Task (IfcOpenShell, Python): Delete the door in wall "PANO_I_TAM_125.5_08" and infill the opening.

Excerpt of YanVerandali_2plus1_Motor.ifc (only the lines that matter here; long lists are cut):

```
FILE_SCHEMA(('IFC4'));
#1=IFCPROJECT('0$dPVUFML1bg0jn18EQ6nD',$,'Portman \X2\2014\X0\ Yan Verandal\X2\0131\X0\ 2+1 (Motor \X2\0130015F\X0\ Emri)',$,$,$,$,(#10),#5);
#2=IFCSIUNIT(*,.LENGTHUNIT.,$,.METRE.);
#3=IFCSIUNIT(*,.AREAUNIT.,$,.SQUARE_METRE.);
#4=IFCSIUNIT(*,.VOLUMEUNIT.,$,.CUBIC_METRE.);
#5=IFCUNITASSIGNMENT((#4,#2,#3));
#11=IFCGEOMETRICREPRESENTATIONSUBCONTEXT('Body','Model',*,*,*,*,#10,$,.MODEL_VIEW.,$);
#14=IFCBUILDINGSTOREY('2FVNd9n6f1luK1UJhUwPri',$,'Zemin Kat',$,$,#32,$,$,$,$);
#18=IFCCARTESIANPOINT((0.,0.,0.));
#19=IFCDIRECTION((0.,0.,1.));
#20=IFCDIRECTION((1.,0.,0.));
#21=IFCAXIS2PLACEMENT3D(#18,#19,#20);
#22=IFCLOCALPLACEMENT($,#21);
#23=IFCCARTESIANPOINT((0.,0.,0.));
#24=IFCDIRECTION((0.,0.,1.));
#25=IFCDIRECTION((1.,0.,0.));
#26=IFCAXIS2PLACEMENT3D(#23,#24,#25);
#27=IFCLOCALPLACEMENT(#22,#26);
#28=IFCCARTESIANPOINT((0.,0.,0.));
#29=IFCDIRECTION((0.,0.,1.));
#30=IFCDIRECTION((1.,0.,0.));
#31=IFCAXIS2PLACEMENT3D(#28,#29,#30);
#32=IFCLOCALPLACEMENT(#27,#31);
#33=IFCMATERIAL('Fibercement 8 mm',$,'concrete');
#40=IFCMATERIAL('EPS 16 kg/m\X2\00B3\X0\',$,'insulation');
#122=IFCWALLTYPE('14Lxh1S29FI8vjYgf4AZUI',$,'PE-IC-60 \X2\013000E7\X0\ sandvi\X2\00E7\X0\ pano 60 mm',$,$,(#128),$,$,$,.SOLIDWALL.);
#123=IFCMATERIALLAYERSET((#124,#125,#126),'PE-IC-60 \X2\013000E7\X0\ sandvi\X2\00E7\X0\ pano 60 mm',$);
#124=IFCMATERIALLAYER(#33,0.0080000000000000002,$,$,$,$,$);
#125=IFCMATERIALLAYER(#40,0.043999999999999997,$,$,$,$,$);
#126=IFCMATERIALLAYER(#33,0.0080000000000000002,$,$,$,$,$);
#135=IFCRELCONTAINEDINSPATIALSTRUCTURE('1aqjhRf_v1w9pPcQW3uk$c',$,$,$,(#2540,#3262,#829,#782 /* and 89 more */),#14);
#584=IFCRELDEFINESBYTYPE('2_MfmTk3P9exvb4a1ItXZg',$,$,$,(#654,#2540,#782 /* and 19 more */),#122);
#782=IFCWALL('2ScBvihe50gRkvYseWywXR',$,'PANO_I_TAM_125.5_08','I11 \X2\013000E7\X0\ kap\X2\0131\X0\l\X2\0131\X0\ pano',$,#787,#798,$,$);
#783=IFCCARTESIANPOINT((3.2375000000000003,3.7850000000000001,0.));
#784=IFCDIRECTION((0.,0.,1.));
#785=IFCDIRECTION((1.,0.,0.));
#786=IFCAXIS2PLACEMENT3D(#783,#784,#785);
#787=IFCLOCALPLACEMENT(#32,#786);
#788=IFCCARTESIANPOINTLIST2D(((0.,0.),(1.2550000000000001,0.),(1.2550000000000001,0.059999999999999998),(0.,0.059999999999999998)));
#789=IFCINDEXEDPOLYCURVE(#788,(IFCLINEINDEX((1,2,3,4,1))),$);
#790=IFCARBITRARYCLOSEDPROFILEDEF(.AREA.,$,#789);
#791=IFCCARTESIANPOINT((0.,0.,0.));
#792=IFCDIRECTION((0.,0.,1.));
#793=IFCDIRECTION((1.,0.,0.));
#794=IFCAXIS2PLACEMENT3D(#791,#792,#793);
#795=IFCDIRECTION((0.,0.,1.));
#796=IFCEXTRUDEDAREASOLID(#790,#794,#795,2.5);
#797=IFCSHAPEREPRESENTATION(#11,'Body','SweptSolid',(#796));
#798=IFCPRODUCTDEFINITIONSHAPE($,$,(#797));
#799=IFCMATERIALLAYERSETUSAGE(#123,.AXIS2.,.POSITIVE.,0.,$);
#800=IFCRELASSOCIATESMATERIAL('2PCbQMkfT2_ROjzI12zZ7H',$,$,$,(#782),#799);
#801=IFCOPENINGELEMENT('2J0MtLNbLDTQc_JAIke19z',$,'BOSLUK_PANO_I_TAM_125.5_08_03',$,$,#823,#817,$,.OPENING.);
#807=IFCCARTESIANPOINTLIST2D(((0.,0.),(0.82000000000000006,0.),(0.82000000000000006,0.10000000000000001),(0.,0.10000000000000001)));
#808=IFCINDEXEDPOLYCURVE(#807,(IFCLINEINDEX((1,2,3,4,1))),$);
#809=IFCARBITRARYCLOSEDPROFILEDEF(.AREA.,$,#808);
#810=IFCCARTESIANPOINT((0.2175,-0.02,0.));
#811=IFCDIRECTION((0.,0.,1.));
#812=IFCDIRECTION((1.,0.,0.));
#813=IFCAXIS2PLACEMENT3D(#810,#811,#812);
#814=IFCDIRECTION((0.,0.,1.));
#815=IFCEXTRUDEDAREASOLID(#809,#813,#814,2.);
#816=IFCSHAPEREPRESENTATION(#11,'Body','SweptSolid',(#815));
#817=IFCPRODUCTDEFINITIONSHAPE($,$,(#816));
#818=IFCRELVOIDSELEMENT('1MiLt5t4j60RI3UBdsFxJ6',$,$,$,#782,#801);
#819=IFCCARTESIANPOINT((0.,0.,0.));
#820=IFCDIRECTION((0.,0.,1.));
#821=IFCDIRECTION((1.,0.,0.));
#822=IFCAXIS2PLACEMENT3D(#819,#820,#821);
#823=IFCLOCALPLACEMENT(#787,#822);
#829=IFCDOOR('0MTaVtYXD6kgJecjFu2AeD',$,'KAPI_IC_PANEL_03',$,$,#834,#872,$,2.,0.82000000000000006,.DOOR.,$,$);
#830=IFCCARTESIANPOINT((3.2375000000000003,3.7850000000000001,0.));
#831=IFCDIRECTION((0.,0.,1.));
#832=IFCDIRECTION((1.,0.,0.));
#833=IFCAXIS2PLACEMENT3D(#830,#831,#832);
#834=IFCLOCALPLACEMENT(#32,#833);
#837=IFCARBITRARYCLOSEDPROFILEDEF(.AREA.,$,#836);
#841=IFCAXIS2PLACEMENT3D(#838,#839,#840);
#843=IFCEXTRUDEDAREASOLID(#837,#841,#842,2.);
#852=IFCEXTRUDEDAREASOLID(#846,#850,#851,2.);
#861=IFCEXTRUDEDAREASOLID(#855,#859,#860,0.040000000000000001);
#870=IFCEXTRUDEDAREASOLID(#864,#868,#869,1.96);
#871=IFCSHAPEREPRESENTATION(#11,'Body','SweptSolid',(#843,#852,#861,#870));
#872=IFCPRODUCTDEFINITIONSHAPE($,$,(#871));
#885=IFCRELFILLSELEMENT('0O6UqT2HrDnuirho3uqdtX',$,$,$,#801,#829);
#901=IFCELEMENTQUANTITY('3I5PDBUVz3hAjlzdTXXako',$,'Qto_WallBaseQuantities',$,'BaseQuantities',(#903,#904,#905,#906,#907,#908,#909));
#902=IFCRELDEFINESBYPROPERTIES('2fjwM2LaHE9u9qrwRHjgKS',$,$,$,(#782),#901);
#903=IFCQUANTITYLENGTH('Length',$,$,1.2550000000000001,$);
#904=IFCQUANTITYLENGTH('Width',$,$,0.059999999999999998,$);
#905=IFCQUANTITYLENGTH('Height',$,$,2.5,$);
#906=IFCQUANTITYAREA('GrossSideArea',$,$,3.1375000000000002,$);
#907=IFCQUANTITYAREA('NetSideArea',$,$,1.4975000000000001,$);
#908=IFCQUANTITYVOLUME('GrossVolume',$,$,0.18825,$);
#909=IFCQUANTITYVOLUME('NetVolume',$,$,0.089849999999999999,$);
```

```python
import ifcopenshell
import ifcopenshell.api.feature
import ifcopenshell.api.pset
import ifcopenshell.api.root
import ifcopenshell.geom
import ifcopenshell.util.element
import ifcopenshell.util.shape
import ifcopenshell.util.unit

model = ifcopenshell.open("YanVerandali_2plus1_Motor.ifc")
area_scale = ifcopenshell.util.unit.calculate_unit_scale(model, "AREAUNIT")
volume_scale = ifcopenshell.util.unit.calculate_unit_scale(model, "VOLUMEUNIT")
settings = ifcopenshell.geom.settings()


def volume(element):
    """Net volume in cubic metres, openings subtracted."""
    shape = ifcopenshell.geom.create_shape(settings, element)
    return ifcopenshell.util.shape.get_volume(shape.geometry)


door = model.by_guid("0MTaVtYXD6kgJecjFu2AeD")
opening = door.FillsVoids[0].RelatingOpeningElement
wall = opening.VoidsElements[0].RelatingBuildingElement
before = volume(wall)

ifcopenshell.api.root.remove_product(model, product=door)
ifcopenshell.api.feature.remove_feature(model, feature=opening)

after = volume(wall)
thickness = 0.06  # wall thickness in metres

# Update the wall's stored quantities.
qto = model.by_id(ifcopenshell.util.element.get_pset(wall, "Qto_WallBaseQuantities", should_inherit=False)["id"])
ifcopenshell.api.pset.edit_qto(model, qto=qto, properties={
    "NetSideArea": after / thickness / area_scale,
    "NetVolume": after / volume_scale,
})

print(f"wall volume {before:.3f} -> {after:.3f} m3")

model.write("YanVerandali_2plus1_Motor_rev.ifc")
```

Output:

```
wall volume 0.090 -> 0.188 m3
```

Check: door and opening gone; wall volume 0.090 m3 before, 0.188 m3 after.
